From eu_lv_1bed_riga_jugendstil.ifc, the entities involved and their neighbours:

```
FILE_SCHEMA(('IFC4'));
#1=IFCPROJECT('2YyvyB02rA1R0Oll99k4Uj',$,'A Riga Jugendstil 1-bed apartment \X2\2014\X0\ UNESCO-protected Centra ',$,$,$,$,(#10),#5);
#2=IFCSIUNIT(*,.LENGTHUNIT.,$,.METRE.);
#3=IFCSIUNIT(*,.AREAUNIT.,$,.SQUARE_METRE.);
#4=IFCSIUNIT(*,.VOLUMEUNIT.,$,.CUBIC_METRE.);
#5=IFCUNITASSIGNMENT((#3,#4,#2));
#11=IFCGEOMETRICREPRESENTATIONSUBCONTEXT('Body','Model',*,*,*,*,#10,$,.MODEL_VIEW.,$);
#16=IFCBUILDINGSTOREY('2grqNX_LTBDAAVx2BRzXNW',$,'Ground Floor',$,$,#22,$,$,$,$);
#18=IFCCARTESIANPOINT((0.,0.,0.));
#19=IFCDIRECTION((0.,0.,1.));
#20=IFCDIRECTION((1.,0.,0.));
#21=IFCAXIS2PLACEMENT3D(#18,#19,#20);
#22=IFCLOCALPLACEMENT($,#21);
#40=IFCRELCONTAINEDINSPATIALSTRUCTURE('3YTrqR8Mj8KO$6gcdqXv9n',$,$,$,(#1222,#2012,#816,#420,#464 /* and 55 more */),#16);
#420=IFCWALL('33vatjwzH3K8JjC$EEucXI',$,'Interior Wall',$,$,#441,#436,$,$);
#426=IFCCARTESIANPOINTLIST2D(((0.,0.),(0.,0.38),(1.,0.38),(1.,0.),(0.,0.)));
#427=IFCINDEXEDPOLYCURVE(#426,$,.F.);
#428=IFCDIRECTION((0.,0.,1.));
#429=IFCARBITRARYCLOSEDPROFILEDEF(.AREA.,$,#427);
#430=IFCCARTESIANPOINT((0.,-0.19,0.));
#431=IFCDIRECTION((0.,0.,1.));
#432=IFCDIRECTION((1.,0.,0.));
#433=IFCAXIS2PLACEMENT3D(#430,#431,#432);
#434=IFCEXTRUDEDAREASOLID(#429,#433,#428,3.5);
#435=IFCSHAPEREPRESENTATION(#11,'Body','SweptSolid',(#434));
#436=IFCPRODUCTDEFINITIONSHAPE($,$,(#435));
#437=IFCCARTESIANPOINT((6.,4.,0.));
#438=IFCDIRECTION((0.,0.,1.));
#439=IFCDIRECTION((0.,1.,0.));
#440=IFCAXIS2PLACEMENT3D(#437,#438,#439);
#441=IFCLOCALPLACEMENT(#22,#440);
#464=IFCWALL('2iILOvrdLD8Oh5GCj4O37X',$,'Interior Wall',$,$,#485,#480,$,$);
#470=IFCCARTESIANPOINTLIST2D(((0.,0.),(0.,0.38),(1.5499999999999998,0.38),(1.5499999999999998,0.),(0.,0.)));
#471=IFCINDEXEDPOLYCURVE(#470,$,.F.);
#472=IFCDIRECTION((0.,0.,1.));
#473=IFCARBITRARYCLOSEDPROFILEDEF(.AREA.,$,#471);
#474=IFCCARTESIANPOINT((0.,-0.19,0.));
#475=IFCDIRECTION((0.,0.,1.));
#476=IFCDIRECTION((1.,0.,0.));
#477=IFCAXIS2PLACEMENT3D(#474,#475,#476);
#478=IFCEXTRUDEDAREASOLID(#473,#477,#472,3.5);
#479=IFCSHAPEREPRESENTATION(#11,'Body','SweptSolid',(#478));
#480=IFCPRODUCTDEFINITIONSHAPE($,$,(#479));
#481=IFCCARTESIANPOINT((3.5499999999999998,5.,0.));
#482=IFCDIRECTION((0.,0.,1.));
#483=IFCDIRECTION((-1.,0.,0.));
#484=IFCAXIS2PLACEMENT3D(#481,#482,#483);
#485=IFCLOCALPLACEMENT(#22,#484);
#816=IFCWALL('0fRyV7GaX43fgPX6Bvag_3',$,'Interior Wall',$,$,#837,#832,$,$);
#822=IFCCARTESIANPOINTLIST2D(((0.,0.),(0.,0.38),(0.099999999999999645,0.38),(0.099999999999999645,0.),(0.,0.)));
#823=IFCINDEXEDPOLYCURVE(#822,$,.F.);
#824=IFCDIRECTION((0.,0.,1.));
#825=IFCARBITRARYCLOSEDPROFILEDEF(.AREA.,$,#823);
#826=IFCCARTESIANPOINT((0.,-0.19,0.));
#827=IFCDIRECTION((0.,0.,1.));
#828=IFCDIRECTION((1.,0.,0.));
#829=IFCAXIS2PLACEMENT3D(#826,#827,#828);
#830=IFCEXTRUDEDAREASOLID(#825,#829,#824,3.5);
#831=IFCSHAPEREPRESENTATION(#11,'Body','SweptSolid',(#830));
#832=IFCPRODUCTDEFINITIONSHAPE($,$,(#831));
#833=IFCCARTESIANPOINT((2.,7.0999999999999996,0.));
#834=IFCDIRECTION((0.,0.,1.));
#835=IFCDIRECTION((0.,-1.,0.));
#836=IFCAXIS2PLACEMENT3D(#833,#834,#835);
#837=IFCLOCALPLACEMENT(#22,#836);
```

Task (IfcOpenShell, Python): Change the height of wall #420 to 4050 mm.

```python
import ifcopenshell
import ifcopenshell.geom
import ifcopenshell.util.representation
import ifcopenshell.util.shape

model = ifcopenshell.open("eu_lv_1bed_riga_jugendstil.ifc")
settings = ifcopenshell.geom.settings()


def volume(element):
    """Net volume in cubic metres, openings subtracted."""
    shape = ifcopenshell.geom.create_shape(settings, element)
    return ifcopenshell.util.shape.get_volume(shape.geometry)


wall = model.by_guid("33vatjwzH3K8JjC$EEucXI")
before = volume(wall)

body = ifcopenshell.util.representation.get_representation(wall, "Model", "Body")
solid = body.Items[0]
old_height = solid.Depth
solid.Depth = 4.05
after = volume(wall)

print(f"height {old_height:g} -> {solid.Depth:g}, volume {before:.3f} -> {after:.3f} m3")

model.write("eu_lv_1bed_riga_jugendstil-out.ifc")
```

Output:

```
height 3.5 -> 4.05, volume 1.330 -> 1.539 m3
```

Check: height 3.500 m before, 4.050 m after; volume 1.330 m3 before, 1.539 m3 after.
